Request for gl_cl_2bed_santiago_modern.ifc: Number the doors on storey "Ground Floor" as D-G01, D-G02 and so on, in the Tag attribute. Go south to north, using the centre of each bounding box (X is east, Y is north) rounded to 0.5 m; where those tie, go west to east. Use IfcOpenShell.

First a look at what the model holds.

```python
import ifcopenshell
import ifcopenshell.util.element
import ifcopenshell.util.placement

model = ifcopenshell.open("gl_cl_2bed_santiago_modern.ifc")
print(model.schema)
storey = next(s for s in model.by_type("IfcBuildingStorey") if s.Name == "Ground Floor")
doors = [e for e in ifcopenshell.util.element.get_decomposition(storey) if e.is_a("IfcDoor")]
for e in sorted(doors, key=lambda e: e.id()):
    origin = ifcopenshell.util.placement.get_local_placement(e.ObjectPlacement)[:3, 3]
    print(e.id(), e.Tag, e.Name, origin.round(2) + 0.0, sep=" | ")
```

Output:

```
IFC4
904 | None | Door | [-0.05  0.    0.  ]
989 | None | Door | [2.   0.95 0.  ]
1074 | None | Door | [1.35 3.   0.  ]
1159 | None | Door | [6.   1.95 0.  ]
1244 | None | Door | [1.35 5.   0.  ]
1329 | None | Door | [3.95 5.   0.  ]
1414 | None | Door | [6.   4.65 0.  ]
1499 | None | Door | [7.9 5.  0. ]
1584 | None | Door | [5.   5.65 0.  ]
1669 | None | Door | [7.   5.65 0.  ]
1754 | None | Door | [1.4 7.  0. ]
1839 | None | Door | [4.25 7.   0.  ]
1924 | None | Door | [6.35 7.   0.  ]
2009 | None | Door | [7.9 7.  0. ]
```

```python
import ifcopenshell
import ifcopenshell.geom
import ifcopenshell.util.element
import ifcopenshell.util.shape

model = ifcopenshell.open("gl_cl_2bed_santiago_modern.ifc")
settings = ifcopenshell.geom.settings()
settings.set("use-world-coords", True)


def centre(element):
    shape = ifcopenshell.geom.create_shape(settings, element)
    return ifcopenshell.util.shape.get_bbox_centroid(shape.geometry)


storey = next(s for s in model.by_type("IfcBuildingStorey") if s.Name == "Ground Floor")
doors = [e for e in ifcopenshell.util.element.get_decomposition(storey) if e.is_a("IfcDoor")]

# Insertion points can sit at a corner or the storey origin, so sort by the geometry (in metres).
centres = {e: centre(e) for e in doors}
doors.sort(key=lambda e: (round(centres[e][1] / 0.5), centres[e][0]))

for i, e in enumerate(doors, start=1):
    number = f"D-G{i:02d}"
    e.Tag = number
    print(e.id(), number)

model.write("gl_cl_2bed_santiago_modern_updated.ifc")
```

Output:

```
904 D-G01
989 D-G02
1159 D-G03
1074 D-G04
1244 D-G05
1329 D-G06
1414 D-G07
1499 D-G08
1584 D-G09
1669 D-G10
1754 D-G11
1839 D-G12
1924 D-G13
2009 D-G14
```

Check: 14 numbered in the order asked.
